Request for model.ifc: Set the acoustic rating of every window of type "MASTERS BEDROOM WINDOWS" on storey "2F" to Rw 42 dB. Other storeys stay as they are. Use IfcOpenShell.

First a look at what the model holds.

```python
import ifcopenshell
import ifcopenshell.util.element

model = ifcopenshell.open("model.ifc")
print(model.schema)
storey = next(s for s in model.by_type("IfcBuildingStorey") if s.Name == "2F")
windows = [e for e in ifcopenshell.util.element.get_decomposition(storey) if e.is_a("IfcWindow")]
seen = {}
for e in windows:
    element_type = ifcopenshell.util.element.get_type(e)
    key = (element_type.Name if element_type != e and element_type else None, ifcopenshell.util.element.get_pset(e, "Pset_WindowCommon", "AcousticRating"))
    seen[key] = seen.get(key, 0) + 1
for (name, value), count in sorted(seen.items(), key=str):
    print(count, "x", name, "|", value)
```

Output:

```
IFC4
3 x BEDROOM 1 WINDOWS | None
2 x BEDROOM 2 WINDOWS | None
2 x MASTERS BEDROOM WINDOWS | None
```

```python
import ifcopenshell
import ifcopenshell.api.pset
import ifcopenshell.util.element

model = ifcopenshell.open("model.ifc")

storey = next(s for s in model.by_type("IfcBuildingStorey") if s.Name == "2F")
windows = [e for e in ifcopenshell.util.element.get_decomposition(storey) if e.is_a("IfcWindow")]

count = 0
for e in windows:
    element_type = ifcopenshell.util.element.get_type(e)
    if element_type in (None, e) or element_type.Name != "MASTERS BEDROOM WINDOWS":
        continue
    # add_pset returns the element's existing set when there is one.
    pset = ifcopenshell.api.pset.add_pset(model, product=e, name="Pset_WindowCommon")
    ifcopenshell.api.pset.edit_pset(model, pset=pset, properties={"AcousticRating": "Rw 42 dB"})
    count += 1

print(count, "windows updated")

model.write("model_updated.ifc")
```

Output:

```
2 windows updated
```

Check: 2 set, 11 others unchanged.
